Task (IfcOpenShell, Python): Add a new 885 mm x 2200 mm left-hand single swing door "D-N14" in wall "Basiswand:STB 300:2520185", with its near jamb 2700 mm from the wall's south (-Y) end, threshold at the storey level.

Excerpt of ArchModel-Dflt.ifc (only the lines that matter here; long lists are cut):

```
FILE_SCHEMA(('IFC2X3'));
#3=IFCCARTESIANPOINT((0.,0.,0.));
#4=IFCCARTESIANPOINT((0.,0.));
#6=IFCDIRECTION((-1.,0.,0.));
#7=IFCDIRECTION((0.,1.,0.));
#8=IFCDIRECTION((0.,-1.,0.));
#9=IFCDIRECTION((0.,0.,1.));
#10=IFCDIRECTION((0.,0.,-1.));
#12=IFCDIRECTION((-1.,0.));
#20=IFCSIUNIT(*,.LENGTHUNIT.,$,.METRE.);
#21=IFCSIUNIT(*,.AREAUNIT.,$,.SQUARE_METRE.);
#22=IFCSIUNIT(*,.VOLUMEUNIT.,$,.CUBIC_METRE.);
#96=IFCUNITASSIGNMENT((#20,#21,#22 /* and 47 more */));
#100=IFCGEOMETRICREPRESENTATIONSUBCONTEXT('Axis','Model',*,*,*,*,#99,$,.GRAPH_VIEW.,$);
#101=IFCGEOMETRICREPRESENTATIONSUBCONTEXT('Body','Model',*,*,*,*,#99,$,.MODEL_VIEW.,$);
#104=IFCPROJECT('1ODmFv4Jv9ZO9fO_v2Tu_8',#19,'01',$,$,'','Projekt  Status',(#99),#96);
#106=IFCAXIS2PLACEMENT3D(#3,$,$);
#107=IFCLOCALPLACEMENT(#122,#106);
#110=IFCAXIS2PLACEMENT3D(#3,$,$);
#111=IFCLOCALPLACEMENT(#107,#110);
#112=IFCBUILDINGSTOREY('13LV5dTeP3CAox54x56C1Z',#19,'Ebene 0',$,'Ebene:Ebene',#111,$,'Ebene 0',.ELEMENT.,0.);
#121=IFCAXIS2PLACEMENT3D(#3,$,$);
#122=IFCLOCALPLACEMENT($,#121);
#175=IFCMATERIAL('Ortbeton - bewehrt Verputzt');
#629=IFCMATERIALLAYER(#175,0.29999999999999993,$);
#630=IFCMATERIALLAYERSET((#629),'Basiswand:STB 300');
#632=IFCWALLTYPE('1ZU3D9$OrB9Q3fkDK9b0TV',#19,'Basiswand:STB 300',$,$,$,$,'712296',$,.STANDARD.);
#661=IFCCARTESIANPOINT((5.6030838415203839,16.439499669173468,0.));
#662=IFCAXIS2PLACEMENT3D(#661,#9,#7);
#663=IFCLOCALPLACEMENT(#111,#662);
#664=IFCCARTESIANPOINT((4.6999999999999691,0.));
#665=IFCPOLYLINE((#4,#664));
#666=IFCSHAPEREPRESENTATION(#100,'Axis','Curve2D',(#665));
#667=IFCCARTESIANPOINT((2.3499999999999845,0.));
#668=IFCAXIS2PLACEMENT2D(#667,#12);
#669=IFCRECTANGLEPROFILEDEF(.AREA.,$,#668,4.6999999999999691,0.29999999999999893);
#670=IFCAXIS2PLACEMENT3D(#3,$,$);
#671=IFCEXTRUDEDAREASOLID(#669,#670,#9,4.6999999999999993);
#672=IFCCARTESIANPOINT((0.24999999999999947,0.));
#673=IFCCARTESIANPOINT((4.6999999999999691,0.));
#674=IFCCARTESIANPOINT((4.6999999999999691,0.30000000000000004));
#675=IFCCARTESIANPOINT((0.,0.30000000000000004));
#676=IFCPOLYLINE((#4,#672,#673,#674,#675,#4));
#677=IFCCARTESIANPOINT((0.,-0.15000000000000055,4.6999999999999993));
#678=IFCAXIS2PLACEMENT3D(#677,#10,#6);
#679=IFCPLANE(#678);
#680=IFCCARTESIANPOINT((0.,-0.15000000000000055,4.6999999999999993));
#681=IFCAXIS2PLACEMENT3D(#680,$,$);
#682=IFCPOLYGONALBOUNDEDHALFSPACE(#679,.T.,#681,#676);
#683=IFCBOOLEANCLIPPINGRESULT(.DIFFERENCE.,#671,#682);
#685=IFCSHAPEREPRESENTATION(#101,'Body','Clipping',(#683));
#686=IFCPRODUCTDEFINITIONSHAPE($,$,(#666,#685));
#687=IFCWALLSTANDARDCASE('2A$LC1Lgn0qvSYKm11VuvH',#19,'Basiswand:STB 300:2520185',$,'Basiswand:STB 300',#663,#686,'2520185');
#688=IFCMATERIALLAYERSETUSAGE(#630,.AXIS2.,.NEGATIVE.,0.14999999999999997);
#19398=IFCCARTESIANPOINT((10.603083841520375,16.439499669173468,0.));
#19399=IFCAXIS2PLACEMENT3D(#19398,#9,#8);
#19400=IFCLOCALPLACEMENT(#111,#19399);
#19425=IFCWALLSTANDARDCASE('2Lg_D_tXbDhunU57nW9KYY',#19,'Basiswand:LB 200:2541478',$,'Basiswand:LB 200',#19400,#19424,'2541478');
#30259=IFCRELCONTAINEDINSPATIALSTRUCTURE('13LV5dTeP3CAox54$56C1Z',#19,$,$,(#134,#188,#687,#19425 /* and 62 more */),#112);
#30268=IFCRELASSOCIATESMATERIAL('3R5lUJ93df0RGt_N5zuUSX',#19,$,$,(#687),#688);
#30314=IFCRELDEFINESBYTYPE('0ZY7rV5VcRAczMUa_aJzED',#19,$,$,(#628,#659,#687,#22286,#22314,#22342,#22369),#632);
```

```python
import numpy as np
import ifcopenshell
import ifcopenshell.api.feature
import ifcopenshell.api.geometry
import ifcopenshell.api.root
import ifcopenshell.api.spatial
import ifcopenshell.api.type
import ifcopenshell.geom
import ifcopenshell.util.element
import ifcopenshell.util.placement
import ifcopenshell.util.representation
import ifcopenshell.util.shape
import ifcopenshell.util.unit

model = ifcopenshell.open("ArchModel-Dflt.ifc")
unit_scale = ifcopenshell.util.unit.calculate_unit_scale(model)
settings = ifcopenshell.geom.settings()


def volume(element):
    """Net volume in cubic metres, openings subtracted."""
    shape = ifcopenshell.geom.create_shape(settings, element)
    return ifcopenshell.util.shape.get_volume(shape.geometry)


wall = model.by_guid("2A$LC1Lgn0qvSYKm11VuvH")
storey = ifcopenshell.util.element.get_container(wall, ifc_class="IfcBuildingStorey")
context = ifcopenshell.util.representation.get_context(model, "Model", "Body", "MODEL_VIEW")
before = volume(wall)

width, height, from_end, sill = 0.885, 2.2, 2.7, 0.0  # metres

# The wall runs along its own X axis, and the end named is its -X end.
wall_shape = ifcopenshell.geom.create_shape(settings, wall)
x, y, z = ifcopenshell.util.shape.get_vertices(wall_shape.geometry).T
start = x.min() + from_end
face, thickness = float(y.min()), float(y.max() - y.min())
wall_matrix = ifcopenshell.util.placement.get_local_placement(wall.ObjectPlacement)
level = ifcopenshell.util.placement.get_local_placement(storey.ObjectPlacement)[2, 3]


def in_wall(x, y):
    """Placement at x, y metres in the wall's axes, at sill height."""
    matrix = wall_matrix.copy()
    matrix[:, 3] = wall_matrix @ np.array([x / unit_scale, y / unit_scale, 0.0, 1.0])
    matrix[2, 3] = level + sill / unit_scale
    return matrix


# Opening: a box that overshoots both wall faces by 50 mm.
opening = ifcopenshell.api.root.create_entity(model, ifc_class="IfcOpeningElement")
box = ifcopenshell.api.geometry.add_wall_representation(
    model, context=context, length=width, height=height, thickness=thickness + 0.1
)
ifcopenshell.api.geometry.assign_representation(model, product=opening, representation=box)
ifcopenshell.api.geometry.edit_object_placement(model, product=opening, matrix=in_wall(start, face - 0.05), is_si=False)
ifcopenshell.api.feature.add_feature(model, feature=opening, element=wall)

door = ifcopenshell.api.root.create_entity(model, ifc_class="IfcDoor", name="D-N14")
door.OverallWidth, door.OverallHeight = width / unit_scale, height / unit_scale
body = ifcopenshell.api.geometry.add_door_representation(
    model,
    context=context,
    overall_width=door.OverallWidth,
    overall_height=door.OverallHeight,
    operation_type="SINGLE_SWING_LEFT",
    lining_properties={"LiningDepth": thickness / unit_scale, "ThresholdDepth": thickness / unit_scale},
)
ifcopenshell.api.geometry.assign_representation(model, product=door, representation=body)
ifcopenshell.api.spatial.assign_container(model, products=[door], relating_structure=storey)
fills = ifcopenshell.api.feature.add_filling(model, opening=opening, element=door)
fills.OwnerHistory = door.OwnerHistory  # required in IFC2X3

# IFC2X3 keeps the operation on the door style.
style = ifcopenshell.api.root.create_entity(model, ifc_class="IfcDoorStyle", name="D-N14")
style.OperationType, style.ConstructionType = "SINGLE_SWING_LEFT", "NOTDEFINED"
style.ParameterTakesPrecedence = style.Sizeable = False
ifcopenshell.api.type.assign_type(model, related_objects=[door], relating_type=style)

# The lining spans the wall, so the door starts at the wall face.
ifcopenshell.api.geometry.edit_object_placement(model, product=door, matrix=in_wall(start, face), is_si=False)

after = volume(wall)

print(f"wall volume {before:.3f} -> {after:.3f} m3")

model.write("ArchModel-Dflt_edited.ifc")
```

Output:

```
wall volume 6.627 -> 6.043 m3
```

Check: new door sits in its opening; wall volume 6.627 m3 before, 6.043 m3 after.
